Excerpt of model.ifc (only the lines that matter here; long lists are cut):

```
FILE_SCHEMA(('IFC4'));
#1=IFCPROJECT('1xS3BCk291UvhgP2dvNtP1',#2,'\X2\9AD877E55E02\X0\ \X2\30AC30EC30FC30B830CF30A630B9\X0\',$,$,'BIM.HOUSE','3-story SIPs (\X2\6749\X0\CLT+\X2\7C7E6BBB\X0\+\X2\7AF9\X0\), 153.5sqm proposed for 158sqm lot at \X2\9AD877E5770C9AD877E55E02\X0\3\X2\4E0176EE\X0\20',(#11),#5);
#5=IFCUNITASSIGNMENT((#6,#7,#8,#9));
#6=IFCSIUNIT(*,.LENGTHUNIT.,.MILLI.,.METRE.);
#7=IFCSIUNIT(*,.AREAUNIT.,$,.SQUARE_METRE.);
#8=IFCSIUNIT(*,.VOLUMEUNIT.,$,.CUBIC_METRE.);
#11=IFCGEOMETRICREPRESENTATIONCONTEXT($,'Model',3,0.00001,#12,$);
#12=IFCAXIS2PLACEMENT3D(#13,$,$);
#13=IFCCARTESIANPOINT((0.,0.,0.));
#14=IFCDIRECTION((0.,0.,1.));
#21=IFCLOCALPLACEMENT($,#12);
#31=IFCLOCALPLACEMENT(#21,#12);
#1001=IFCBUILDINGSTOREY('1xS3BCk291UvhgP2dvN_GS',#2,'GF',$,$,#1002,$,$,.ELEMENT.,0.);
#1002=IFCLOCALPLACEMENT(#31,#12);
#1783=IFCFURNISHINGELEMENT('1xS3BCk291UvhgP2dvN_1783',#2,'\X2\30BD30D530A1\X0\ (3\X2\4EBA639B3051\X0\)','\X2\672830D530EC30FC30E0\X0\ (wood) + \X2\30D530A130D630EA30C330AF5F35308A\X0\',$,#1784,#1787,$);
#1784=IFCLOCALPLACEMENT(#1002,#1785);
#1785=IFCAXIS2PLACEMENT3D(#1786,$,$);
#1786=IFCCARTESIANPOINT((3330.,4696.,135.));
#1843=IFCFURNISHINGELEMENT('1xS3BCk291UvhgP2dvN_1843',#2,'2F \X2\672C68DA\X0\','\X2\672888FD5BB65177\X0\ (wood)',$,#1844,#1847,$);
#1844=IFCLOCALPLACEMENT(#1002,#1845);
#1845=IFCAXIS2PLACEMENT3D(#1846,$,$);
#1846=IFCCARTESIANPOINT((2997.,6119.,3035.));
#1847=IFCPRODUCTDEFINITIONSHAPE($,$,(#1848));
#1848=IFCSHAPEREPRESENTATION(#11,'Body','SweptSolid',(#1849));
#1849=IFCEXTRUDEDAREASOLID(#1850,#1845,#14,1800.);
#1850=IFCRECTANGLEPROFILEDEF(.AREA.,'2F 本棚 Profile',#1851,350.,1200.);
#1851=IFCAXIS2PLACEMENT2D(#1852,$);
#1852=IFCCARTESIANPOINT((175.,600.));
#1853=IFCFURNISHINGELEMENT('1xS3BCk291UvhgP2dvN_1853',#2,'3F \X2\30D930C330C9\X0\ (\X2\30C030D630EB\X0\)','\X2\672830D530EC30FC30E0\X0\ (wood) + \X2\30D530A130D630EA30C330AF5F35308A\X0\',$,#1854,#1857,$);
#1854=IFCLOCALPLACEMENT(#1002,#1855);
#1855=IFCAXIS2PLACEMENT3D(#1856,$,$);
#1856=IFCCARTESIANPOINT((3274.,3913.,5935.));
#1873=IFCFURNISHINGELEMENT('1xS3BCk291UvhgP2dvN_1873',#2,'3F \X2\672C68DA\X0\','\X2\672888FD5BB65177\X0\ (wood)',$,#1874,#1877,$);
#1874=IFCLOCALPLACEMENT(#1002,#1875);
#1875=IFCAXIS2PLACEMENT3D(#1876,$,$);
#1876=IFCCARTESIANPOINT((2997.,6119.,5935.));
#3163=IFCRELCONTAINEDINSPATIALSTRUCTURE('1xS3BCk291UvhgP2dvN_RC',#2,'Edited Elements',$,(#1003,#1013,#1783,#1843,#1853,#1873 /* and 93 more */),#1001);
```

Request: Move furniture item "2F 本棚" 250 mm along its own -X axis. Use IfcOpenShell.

```python
import ifcopenshell
import ifcopenshell.api.geometry
import ifcopenshell.util.placement
import ifcopenshell.util.unit

model = ifcopenshell.open("model.ifc")
unit_scale = ifcopenshell.util.unit.calculate_unit_scale(model)

item = model.by_id(1843)
matrix = ifcopenshell.util.placement.get_local_placement(item.ObjectPlacement)
matrix[:3, 3] -= matrix[:3, 0] * 0.25 / unit_scale
ifcopenshell.api.geometry.edit_object_placement(model, product=item, matrix=matrix, is_si=False)

print(ifcopenshell.util.placement.get_local_placement(item.ObjectPlacement).round(3) + 0.0)

model.write("model_v2.ifc")
```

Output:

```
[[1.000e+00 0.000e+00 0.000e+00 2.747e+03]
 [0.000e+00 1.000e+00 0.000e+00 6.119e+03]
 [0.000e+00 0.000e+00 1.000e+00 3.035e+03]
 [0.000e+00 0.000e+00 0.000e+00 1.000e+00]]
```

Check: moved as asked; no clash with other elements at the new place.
